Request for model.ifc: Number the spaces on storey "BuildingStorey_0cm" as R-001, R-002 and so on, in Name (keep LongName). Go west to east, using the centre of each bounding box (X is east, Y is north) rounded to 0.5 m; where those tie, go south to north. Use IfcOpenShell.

First a look at what the model holds.

```python
import ifcopenshell
import ifcopenshell.util.element
import ifcopenshell.util.placement

model = ifcopenshell.open("model.ifc")
print(model.schema)
storey = next(s for s in model.by_type("IfcBuildingStorey") if s.Name == "BuildingStorey_0cm")
spaces = [e for e in ifcopenshell.util.element.get_decomposition(storey) if e.is_a("IfcSpace")]
for e in sorted(spaces, key=lambda e: e.id()):
    origin = ifcopenshell.util.placement.get_local_placement(e.ObjectPlacement)[:3, 3]
    print(e.id(), e.Name, e.LongName, origin.round(2) + 0.0, sep=" | ")
```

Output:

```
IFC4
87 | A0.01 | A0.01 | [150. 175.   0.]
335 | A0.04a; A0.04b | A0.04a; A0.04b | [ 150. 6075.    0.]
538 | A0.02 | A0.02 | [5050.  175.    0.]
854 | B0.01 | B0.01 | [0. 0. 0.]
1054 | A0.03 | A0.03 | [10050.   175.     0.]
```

```python
import ifcopenshell
import ifcopenshell.geom
import ifcopenshell.util.element
import ifcopenshell.util.shape

model = ifcopenshell.open("model.ifc")
settings = ifcopenshell.geom.settings()
settings.set("use-world-coords", True)


def centre(element):
    shape = ifcopenshell.geom.create_shape(settings, element)
    return ifcopenshell.util.shape.get_bbox_centroid(shape.geometry)


storey = next(s for s in model.by_type("IfcBuildingStorey") if s.Name == "BuildingStorey_0cm")
spaces = [e for e in ifcopenshell.util.element.get_decomposition(storey) if e.is_a("IfcSpace")]

# Insertion points can sit at a corner or the storey origin, so sort by the geometry (in metres).
centres = {e: centre(e) for e in spaces}
spaces.sort(key=lambda e: (round(centres[e][0] / 0.5), centres[e][1]))

for i, e in enumerate(spaces, start=1):
    number = f"R-0{i:02d}"
    e.Name = number
    print(e.id(), number)

model.write("model_updated.ifc")
```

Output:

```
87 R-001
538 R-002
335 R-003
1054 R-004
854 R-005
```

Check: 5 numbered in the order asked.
